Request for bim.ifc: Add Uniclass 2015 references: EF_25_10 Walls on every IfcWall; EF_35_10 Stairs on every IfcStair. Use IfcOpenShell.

First a look at what the model holds.

```python
import ifcopenshell

model = ifcopenshell.open("bim.ifc")
print(model.schema)
print("classifications:", [c.Name for c in model.by_type("IfcClassification")])
for ifc_class in ("IfcDoor", "IfcRoof", "IfcStair", "IfcWall", "IfcWindow"):
    print(ifc_class, len(model.by_type(ifc_class)))
```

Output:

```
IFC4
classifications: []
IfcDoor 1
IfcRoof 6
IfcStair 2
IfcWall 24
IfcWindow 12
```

```python
import ifcopenshell
import ifcopenshell.api.classification

model = ifcopenshell.open("bim.ifc")

system = ifcopenshell.api.classification.add_classification(model, classification="Uniclass 2015")

codes = {
    "IfcWall": ("EF_25_10", "Walls"),
    "IfcStair": ("EF_35_10", "Stairs"),
}
for ifc_class, (code, name) in codes.items():
    products = model.by_type(ifc_class)
    ifcopenshell.api.classification.add_reference(
        model, products=products, classification=system, identification=code, name=name
    )
    print(code, len(products))

model.write("bim_edited.ifc")
```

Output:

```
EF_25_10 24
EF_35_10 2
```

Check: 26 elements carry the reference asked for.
